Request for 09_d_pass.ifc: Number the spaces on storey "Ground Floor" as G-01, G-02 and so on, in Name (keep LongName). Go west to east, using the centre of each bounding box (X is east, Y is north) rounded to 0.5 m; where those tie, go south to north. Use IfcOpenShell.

First a look at what the model holds.

```python
import ifcopenshell
import ifcopenshell.util.element
import ifcopenshell.util.placement

model = ifcopenshell.open("09_d_pass.ifc")
print(model.schema)
storey = next(s for s in model.by_type("IfcBuildingStorey") if s.Name == "Ground Floor")
spaces = [e for e in ifcopenshell.util.element.get_decomposition(storey) if e.is_a("IfcSpace")]
for e in sorted(spaces, key=lambda e: e.id()):
    origin = ifcopenshell.util.placement.get_local_placement(e.ObjectPlacement)[:3, 3]
    print(e.id(), e.Name, e.LongName, origin.round(2) + 0.0, sep=" | ")
```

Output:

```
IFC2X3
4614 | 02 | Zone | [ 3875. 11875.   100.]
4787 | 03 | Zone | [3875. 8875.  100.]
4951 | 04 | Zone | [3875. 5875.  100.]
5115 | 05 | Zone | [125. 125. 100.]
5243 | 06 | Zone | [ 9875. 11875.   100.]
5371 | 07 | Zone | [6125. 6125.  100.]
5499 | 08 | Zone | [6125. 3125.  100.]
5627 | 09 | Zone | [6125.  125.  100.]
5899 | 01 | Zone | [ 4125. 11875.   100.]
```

```python
import ifcopenshell
import ifcopenshell.geom
import ifcopenshell.util.element
import ifcopenshell.util.shape

model = ifcopenshell.open("09_d_pass.ifc")
settings = ifcopenshell.geom.settings()
settings.set("use-world-coords", True)


def centre(element):
    shape = ifcopenshell.geom.create_shape(settings, element)
    return ifcopenshell.util.shape.get_bbox_centroid(shape.geometry)


storey = next(s for s in model.by_type("IfcBuildingStorey") if s.Name == "Ground Floor")
spaces = [e for e in ifcopenshell.util.element.get_decomposition(storey) if e.is_a("IfcSpace")]

# Insertion points can sit at a corner or the storey origin, so sort by the geometry (in metres).
centres = {e: centre(e) for e in spaces}
spaces.sort(key=lambda e: (round(centres[e][0] / 0.5), centres[e][1]))

for i, e in enumerate(spaces, start=1):
    number = f"G-{i:02d}"
    e.Name = number
    print(e.id(), number)

model.write("09_d_pass_updated.ifc")
```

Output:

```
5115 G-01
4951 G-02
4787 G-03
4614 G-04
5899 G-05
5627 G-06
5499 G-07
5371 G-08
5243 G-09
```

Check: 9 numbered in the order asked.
